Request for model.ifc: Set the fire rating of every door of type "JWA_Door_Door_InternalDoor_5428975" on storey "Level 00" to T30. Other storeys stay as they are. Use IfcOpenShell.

First a look at what the model holds.

```python
import ifcopenshell
import ifcopenshell.util.element

model = ifcopenshell.open("model.ifc")
print(model.schema)
storey = next(s for s in model.by_type("IfcBuildingStorey") if s.Name == "Level 00")
doors = [e for e in ifcopenshell.util.element.get_decomposition(storey) if e.is_a("IfcDoor")]
seen = {}
for e in doors:
    element_type = ifcopenshell.util.element.get_type(e)
    key = (element_type.Name if element_type != e and element_type else None, ifcopenshell.util.element.get_pset(e, "Pset_DoorCommon", "FireRating"))
    seen[key] = seen.get(key, 0) + 1
for (name, value), count in sorted(seen.items(), key=str):
    print(count, "x", name, "|", value)
```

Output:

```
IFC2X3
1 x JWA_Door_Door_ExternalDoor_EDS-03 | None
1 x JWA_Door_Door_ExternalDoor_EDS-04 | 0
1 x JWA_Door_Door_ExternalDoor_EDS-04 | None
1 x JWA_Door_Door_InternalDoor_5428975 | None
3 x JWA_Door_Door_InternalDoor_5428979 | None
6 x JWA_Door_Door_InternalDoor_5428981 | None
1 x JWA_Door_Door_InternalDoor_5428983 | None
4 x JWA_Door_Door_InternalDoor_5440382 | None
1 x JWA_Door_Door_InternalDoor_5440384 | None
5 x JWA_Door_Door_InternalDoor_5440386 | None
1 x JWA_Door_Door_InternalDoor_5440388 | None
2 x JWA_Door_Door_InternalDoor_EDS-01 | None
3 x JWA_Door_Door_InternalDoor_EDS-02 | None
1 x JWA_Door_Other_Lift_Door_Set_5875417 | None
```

```python
import ifcopenshell
import ifcopenshell.api.pset
import ifcopenshell.util.element

model = ifcopenshell.open("model.ifc")

storey = next(s for s in model.by_type("IfcBuildingStorey") if s.Name == "Level 00")
doors = [e for e in ifcopenshell.util.element.get_decomposition(storey) if e.is_a("IfcDoor")]

count = 0
for e in doors:
    element_type = ifcopenshell.util.element.get_type(e)
    if element_type in (None, e) or element_type.Name != "JWA_Door_Door_InternalDoor_5428975":
        continue
    # add_pset returns the element's existing set when there is one.
    pset = ifcopenshell.api.pset.add_pset(model, product=e, name="Pset_DoorCommon")
    ifcopenshell.api.pset.edit_pset(model, pset=pset, properties={"FireRating": "T30"})
    count += 1

print(count, "doors updated")

model.write("model_v2.ifc")
```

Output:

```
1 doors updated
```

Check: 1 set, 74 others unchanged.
